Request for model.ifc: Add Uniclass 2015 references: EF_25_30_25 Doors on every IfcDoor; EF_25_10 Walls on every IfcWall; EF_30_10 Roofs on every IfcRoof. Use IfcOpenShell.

First a look at what the model holds.

```python
import ifcopenshell

model = ifcopenshell.open("model.ifc")
print(model.schema)
print("classifications:", [c.Name for c in model.by_type("IfcClassification")])
for ifc_class in ("IfcDoor", "IfcRoof", "IfcStair", "IfcWall", "IfcWindow"):
    print(ifc_class, len(model.by_type(ifc_class)))
```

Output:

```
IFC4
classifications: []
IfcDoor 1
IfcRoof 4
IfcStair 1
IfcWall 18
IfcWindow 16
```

```python
import ifcopenshell
import ifcopenshell.api.classification

model = ifcopenshell.open("model.ifc")

system = ifcopenshell.api.classification.add_classification(model, classification="Uniclass 2015")

codes = {
    "IfcDoor": ("EF_25_30_25", "Doors"),
    "IfcWall": ("EF_25_10", "Walls"),
    "IfcRoof": ("EF_30_10", "Roofs"),
}
for ifc_class, (code, name) in codes.items():
    products = model.by_type(ifc_class)
    ifcopenshell.api.classification.add_reference(
        model, products=products, classification=system, identification=code, name=name
    )
    print(code, len(products))

model.write("model_rev.ifc")
```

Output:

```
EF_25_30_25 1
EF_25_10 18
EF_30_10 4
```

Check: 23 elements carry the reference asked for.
